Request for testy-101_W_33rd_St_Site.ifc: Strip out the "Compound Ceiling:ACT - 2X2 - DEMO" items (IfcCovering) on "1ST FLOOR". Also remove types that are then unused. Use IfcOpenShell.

First a look at what the model holds.

```python
import ifcopenshell
import ifcopenshell.util.element

model = ifcopenshell.open("testy-101_W_33rd_St_Site.ifc")
print(model.schema)
storey = next(s for s in model.by_type("IfcBuildingStorey") if s.Name == "1ST FLOOR")
coverings = [e for e in ifcopenshell.util.element.get_decomposition(storey) if e.is_a("IfcCovering")]
seen = {}
for e in coverings:
    element_type = ifcopenshell.util.element.get_type(e)
    name = element_type.Name if element_type not in (None, e) else None
    seen[name] = seen.get(name, 0) + 1
for name, count in sorted(seen.items(), key=str):
    print(count, "x", name)
```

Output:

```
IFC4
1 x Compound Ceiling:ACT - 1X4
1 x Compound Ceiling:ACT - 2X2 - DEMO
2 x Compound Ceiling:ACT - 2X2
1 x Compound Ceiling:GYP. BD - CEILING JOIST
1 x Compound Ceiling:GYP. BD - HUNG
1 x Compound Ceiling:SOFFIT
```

```python
import ifcopenshell
import ifcopenshell.api.root
import ifcopenshell.util.element

model = ifcopenshell.open("testy-101_W_33rd_St_Site.ifc")

storey = next(s for s in model.by_type("IfcBuildingStorey") if s.Name == "1ST FLOOR")
coverings = [e for e in ifcopenshell.util.element.get_decomposition(storey) if e.is_a("IfcCovering")]
targets = [e for e in coverings if (t := ifcopenshell.util.element.get_type(e)) not in (None, e) and t.Name == "Compound Ceiling:ACT - 2X2 - DEMO"]
types = {ifcopenshell.util.element.get_type(e) for e in targets} - {None, *targets}

for e in targets:
    ifcopenshell.api.root.remove_product(model, product=e)
print(len(targets), "removed")

unused = [t for t in types if not ifcopenshell.util.element.get_types(t)]
for t in unused:
    ifcopenshell.api.root.remove_product(model, product=t)
print(len(unused), "unused types removed")

model.write("testy-101_W_33rd_St_Site_v2.ifc")
```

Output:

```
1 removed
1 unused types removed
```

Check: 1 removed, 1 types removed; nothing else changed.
